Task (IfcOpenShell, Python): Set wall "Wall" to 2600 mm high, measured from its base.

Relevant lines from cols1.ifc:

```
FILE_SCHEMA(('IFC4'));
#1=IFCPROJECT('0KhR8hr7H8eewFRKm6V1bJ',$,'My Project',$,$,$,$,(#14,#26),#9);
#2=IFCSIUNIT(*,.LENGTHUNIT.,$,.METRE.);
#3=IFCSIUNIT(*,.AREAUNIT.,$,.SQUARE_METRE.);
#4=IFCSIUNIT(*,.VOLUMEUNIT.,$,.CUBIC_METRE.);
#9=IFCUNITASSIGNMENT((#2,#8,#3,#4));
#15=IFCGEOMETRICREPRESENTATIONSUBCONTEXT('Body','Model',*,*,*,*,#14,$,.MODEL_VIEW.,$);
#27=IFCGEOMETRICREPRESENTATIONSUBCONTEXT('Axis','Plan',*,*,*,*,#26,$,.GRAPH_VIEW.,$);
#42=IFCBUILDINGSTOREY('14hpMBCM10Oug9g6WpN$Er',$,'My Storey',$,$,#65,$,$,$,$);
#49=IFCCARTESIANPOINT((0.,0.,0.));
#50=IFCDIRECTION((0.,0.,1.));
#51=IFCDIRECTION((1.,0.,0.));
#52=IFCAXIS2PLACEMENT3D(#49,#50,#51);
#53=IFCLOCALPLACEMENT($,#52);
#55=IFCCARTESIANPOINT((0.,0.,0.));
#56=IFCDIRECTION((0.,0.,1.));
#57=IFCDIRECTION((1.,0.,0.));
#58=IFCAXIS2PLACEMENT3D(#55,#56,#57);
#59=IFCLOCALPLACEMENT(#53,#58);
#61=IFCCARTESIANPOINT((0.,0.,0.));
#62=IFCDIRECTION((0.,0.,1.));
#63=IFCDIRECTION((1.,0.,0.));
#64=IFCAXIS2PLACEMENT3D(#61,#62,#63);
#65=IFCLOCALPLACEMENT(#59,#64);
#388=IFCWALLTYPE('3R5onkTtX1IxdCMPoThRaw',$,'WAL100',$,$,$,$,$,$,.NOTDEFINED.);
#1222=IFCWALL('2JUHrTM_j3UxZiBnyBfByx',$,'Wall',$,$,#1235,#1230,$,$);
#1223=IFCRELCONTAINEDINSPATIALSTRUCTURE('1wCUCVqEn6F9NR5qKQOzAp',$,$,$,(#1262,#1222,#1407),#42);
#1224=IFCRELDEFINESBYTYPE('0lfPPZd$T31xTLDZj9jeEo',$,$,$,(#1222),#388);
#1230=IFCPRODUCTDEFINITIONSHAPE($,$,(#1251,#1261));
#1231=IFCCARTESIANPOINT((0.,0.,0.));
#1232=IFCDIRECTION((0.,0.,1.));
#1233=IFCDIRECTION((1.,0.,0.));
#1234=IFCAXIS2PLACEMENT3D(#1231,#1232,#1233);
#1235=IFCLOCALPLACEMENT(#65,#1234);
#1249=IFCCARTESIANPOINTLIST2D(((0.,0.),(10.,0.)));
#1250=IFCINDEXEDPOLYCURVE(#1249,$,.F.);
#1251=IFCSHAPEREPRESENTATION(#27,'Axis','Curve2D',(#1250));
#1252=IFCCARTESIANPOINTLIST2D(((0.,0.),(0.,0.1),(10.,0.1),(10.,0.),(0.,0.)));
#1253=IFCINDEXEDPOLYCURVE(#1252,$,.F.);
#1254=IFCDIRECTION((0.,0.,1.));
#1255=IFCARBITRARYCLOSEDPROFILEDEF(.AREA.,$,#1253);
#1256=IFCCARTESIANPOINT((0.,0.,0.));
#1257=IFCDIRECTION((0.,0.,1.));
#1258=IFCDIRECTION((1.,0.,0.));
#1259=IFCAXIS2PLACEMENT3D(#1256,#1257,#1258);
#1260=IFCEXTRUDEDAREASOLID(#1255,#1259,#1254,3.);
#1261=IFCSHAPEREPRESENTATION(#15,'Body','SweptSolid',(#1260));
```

```python
import ifcopenshell
import ifcopenshell.geom
import ifcopenshell.util.representation
import ifcopenshell.util.shape
import ifcopenshell.util.unit

model = ifcopenshell.open("cols1.ifc")
unit_scale = ifcopenshell.util.unit.calculate_unit_scale(model)
settings = ifcopenshell.geom.settings()


def volume(element):
    """Net volume in cubic metres, openings subtracted."""
    shape = ifcopenshell.geom.create_shape(settings, element)
    return ifcopenshell.util.shape.get_volume(shape.geometry)


wall = model.by_guid("2JUHrTM_j3UxZiBnyBfByx")
before = volume(wall)

body = ifcopenshell.util.representation.get_representation(wall, "Model", "Body")
solid = body.Items[0]
old_height = solid.Depth
solid.Depth = 2.6 / unit_scale
after = volume(wall)

print(f"height {old_height:g} -> {solid.Depth:g}, volume {before:.3f} -> {after:.3f} m3")

model.write("cols1_v2.ifc")
```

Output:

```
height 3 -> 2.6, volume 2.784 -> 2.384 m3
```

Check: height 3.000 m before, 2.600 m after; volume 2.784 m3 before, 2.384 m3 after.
